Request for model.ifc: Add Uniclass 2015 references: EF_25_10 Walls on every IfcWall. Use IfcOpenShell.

First a look at what the model holds.

```python
import ifcopenshell

model = ifcopenshell.open("model.ifc")
print(model.schema)
print("classifications:", [c.Name for c in model.by_type("IfcClassification")])
for ifc_class in ("IfcDoor", "IfcRoof", "IfcStair", "IfcWall", "IfcWindow"):
    print(ifc_class, len(model.by_type(ifc_class)))
```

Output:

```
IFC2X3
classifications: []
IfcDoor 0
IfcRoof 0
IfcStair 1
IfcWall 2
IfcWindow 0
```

```python
import ifcopenshell
import ifcopenshell.api.classification

model = ifcopenshell.open("model.ifc")

# IFC2X3 requires Source and Edition and has no link from the project to the system.
system = model.create_entity("IfcClassification", Source="NBS", Edition="2015", Name="Uniclass 2015")

codes = {
    "IfcWall": ("EF_25_10", "Walls"),
}
for ifc_class, (code, name) in codes.items():
    products = model.by_type(ifc_class)
    ifcopenshell.api.classification.add_reference(
        model, products=products, classification=system, identification=code, name=name
    )
    print(code, len(products))

model.write("model_edited.ifc")
```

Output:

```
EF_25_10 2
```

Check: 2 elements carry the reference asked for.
